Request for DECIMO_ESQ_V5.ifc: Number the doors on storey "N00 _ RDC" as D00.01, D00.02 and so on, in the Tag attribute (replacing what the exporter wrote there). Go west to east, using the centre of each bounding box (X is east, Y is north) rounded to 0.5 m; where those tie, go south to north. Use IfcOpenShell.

First a look at what the model holds.

```python
import ifcopenshell
import ifcopenshell.util.element
import ifcopenshell.util.placement

model = ifcopenshell.open("DECIMO_ESQ_V5.ifc")
print(model.schema)
storey = next(s for s in model.by_type("IfcBuildingStorey") if s.Name == "N00 _ RDC")
doors = [e for e in ifcopenshell.util.element.get_decomposition(storey) if e.is_a("IfcDoor")]
for e in sorted(doors, key=lambda e: e.id()):
    origin = ifcopenshell.util.placement.get_local_placement(e.ObjectPlacement)[:3, 3]
    print(e.id(), e.Tag, e.Name, origin.round(2) + 0.0, sep=" | ")
```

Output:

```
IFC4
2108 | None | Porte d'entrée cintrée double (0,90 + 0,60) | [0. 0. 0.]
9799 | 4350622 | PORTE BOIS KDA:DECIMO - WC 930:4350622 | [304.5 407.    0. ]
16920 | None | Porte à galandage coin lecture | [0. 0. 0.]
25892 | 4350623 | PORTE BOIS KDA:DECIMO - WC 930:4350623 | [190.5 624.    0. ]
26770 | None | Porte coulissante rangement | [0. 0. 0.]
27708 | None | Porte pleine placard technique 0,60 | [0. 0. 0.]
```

```python
import ifcopenshell
import ifcopenshell.geom
import ifcopenshell.util.element
import ifcopenshell.util.shape

model = ifcopenshell.open("DECIMO_ESQ_V5.ifc")
settings = ifcopenshell.geom.settings()
settings.set("use-world-coords", True)


def centre(element):
    shape = ifcopenshell.geom.create_shape(settings, element)
    return ifcopenshell.util.shape.get_bbox_centroid(shape.geometry)


storey = next(s for s in model.by_type("IfcBuildingStorey") if s.Name == "N00 _ RDC")
doors = [e for e in ifcopenshell.util.element.get_decomposition(storey) if e.is_a("IfcDoor")]

# Insertion points can sit at a corner or the storey origin, so sort by the geometry (in metres).
centres = {e: centre(e) for e in doors}
doors.sort(key=lambda e: (round(centres[e][0] / 0.5), centres[e][1]))

for i, e in enumerate(doors, start=1):
    number = f"D00.{i:02d}"
    e.Tag = number
    print(e.id(), number)

model.write("DECIMO_ESQ_V5_edited.ifc")
```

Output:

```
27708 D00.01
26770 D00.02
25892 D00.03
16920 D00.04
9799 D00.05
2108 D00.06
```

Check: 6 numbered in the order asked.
